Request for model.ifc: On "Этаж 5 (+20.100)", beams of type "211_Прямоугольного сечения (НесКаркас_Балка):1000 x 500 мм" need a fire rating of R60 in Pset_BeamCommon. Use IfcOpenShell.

First a look at what the model holds.

```python
import ifcopenshell
import ifcopenshell.util.element

model = ifcopenshell.open("model.ifc")
print(model.schema)
storey = next(s for s in model.by_type("IfcBuildingStorey") if s.Name == "Этаж 5 (+20.100)")
beams = [e for e in ifcopenshell.util.element.get_decomposition(storey) if e.is_a("IfcBeam")]
seen = {}
for e in beams:
    element_type = ifcopenshell.util.element.get_type(e)
    key = (element_type.Name if element_type != e and element_type else None, ifcopenshell.util.element.get_pset(e, "Pset_BeamCommon", "FireRating"))
    seen[key] = seen.get(key, 0) + 1
for (name, value), count in sorted(seen.items(), key=str):
    print(count, "x", name, "|", value)
```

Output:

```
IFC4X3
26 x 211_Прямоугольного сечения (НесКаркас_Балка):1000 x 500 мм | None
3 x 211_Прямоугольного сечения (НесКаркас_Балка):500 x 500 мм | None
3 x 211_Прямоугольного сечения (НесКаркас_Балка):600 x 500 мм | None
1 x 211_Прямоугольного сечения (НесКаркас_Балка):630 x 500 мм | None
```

```python
import ifcopenshell
import ifcopenshell.api.pset
import ifcopenshell.util.element

model = ifcopenshell.open("model.ifc")

storey = next(s for s in model.by_type("IfcBuildingStorey") if s.Name == "Этаж 5 (+20.100)")
beams = [e for e in ifcopenshell.util.element.get_decomposition(storey) if e.is_a("IfcBeam")]

count = 0
for e in beams:
    element_type = ifcopenshell.util.element.get_type(e)
    if element_type in (None, e) or element_type.Name != "211_Прямоугольного сечения (НесКаркас_Балка):1000 x 500 мм":
        continue
    # add_pset returns the element's existing set when there is one.
    pset = ifcopenshell.api.pset.add_pset(model, product=e, name="Pset_BeamCommon")
    ifcopenshell.api.pset.edit_pset(model, pset=pset, properties={"FireRating": "R60"})
    count += 1

print(count, "beams updated")

model.write("model_v2.ifc")
```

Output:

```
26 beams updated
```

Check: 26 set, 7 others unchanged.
